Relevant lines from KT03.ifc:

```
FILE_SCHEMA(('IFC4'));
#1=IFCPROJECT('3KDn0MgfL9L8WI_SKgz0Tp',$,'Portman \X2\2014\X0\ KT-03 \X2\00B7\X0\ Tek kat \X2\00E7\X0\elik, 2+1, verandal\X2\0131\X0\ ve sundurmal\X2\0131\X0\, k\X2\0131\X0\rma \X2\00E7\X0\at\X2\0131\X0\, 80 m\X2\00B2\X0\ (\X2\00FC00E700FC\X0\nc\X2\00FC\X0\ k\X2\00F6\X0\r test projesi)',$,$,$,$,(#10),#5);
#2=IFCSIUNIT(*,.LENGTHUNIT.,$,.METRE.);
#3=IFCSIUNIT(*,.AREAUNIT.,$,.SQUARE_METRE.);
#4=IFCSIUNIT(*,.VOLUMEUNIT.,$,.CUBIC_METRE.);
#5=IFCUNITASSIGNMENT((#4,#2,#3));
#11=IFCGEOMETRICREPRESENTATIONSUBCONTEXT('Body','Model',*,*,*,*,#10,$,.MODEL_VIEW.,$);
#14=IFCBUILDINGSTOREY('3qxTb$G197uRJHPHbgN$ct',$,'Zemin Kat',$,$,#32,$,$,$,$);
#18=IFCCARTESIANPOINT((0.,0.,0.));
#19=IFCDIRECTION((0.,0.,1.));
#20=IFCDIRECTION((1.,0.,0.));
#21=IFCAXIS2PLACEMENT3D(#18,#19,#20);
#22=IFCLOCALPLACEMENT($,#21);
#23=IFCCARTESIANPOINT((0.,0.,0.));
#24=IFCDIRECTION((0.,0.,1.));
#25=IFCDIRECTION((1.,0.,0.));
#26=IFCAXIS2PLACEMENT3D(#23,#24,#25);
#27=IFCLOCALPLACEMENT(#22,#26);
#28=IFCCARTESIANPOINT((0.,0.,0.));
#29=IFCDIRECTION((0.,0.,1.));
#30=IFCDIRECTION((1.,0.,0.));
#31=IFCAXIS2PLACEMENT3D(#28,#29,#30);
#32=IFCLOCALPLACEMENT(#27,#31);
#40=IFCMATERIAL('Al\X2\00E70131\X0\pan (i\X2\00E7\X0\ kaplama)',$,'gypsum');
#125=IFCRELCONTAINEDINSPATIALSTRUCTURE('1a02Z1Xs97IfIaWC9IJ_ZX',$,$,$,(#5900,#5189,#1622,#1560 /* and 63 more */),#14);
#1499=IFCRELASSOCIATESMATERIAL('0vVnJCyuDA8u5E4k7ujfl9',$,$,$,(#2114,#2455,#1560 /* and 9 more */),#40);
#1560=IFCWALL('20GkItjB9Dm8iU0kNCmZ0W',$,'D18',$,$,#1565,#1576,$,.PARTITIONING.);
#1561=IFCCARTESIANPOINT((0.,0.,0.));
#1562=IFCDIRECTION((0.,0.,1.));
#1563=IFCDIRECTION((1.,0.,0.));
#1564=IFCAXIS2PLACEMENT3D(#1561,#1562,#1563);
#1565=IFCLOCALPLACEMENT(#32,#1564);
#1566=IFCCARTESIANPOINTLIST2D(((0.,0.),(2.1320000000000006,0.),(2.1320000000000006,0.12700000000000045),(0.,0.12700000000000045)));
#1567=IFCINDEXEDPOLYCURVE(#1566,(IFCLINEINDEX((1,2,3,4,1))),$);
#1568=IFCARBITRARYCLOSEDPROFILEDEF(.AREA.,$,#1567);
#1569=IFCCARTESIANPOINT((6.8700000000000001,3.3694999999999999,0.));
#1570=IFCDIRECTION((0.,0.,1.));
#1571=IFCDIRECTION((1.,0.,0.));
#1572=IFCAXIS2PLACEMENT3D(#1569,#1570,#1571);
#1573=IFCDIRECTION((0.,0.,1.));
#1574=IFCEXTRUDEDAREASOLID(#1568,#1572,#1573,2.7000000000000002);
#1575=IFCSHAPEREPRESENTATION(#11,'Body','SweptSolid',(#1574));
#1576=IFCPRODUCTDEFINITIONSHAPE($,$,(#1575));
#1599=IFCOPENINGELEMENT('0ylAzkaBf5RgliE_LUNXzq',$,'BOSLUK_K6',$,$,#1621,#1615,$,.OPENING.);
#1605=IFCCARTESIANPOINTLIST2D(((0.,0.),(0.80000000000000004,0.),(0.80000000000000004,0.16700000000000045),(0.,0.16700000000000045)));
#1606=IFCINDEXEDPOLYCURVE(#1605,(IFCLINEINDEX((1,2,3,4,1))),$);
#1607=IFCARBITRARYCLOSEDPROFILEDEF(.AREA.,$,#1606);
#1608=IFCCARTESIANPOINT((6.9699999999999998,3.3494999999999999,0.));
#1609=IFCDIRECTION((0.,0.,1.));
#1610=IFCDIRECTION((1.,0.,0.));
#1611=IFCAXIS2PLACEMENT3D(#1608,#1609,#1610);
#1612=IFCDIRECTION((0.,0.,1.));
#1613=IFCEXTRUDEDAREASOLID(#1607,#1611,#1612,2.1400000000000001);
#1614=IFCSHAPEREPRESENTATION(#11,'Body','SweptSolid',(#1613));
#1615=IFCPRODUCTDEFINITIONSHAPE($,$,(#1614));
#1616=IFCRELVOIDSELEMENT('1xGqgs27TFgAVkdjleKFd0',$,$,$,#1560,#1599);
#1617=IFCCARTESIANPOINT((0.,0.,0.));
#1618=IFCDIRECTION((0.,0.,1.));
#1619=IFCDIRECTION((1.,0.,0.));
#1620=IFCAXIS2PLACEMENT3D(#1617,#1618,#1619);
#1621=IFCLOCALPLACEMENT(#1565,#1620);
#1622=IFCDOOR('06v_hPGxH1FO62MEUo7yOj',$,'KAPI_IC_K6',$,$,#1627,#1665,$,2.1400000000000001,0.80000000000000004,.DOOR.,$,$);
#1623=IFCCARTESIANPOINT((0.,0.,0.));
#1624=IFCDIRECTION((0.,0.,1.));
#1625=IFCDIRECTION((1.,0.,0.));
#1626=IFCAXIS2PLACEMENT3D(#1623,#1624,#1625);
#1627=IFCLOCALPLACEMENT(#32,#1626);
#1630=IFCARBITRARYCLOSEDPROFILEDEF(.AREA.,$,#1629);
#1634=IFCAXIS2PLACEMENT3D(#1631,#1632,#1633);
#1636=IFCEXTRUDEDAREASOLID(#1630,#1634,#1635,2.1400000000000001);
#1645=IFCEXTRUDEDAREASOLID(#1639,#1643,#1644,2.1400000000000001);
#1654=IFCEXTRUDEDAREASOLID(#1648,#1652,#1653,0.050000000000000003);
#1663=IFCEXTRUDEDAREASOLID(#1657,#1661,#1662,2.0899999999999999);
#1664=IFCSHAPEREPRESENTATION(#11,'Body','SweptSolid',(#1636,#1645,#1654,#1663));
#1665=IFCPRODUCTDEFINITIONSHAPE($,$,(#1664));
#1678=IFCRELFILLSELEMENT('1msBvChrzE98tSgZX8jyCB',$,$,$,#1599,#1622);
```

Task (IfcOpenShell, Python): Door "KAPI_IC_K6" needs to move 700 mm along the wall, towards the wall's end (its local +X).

```python
import ifcopenshell
import ifcopenshell.api.geometry
import ifcopenshell.util.placement
import ifcopenshell.util.unit

model = ifcopenshell.open("KT03.ifc")
unit_scale = ifcopenshell.util.unit.calculate_unit_scale(model)

door = model.by_id(1622)
opening = door.FillsVoids[0].RelatingOpeningElement
wall = opening.VoidsElements[0].RelatingBuildingElement

wall_matrix = ifcopenshell.util.placement.get_local_placement(wall.ObjectPlacement)
shift = wall_matrix[:3, 0] * 0.7 / unit_scale
before = ifcopenshell.util.placement.get_local_placement(door.ObjectPlacement)[:3, 3].copy()

# The door is not placed relative to its opening, so move both.
for product in (opening, door):
    matrix = ifcopenshell.util.placement.get_local_placement(product.ObjectPlacement)
    matrix[:3, 3] += shift
    ifcopenshell.api.geometry.edit_object_placement(model, product=product, matrix=matrix, is_si=False)

after = ifcopenshell.util.placement.get_local_placement(door.ObjectPlacement)[:3, 3]
print("door moved by", (after - before).round(3) + 0.0)

model.write("KT03-out.ifc")
```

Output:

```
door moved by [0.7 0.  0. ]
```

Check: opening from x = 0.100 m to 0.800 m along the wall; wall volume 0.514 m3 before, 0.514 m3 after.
